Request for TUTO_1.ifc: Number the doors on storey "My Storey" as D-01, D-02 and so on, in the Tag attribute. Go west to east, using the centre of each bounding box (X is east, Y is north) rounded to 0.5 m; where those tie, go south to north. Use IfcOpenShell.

First a look at what the model holds.

```python
import ifcopenshell
import ifcopenshell.util.element
import ifcopenshell.util.placement

model = ifcopenshell.open("TUTO_1.ifc")
print(model.schema)
storey = next(s for s in model.by_type("IfcBuildingStorey") if s.Name == "My Storey")
doors = [e for e in ifcopenshell.util.element.get_decomposition(storey) if e.is_a("IfcDoor")]
for e in sorted(doors, key=lambda e: e.id()):
    origin = ifcopenshell.util.placement.get_local_placement(e.ObjectPlacement)[:3, 3]
    print(e.id(), e.Tag, e.Name, origin.round(2) + 0.0, sep=" | ")
```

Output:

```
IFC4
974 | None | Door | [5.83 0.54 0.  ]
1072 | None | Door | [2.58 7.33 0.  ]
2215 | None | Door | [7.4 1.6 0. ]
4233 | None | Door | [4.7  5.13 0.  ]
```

```python
import ifcopenshell
import ifcopenshell.geom
import ifcopenshell.util.element
import ifcopenshell.util.shape

model = ifcopenshell.open("TUTO_1.ifc")
settings = ifcopenshell.geom.settings()
settings.set("use-world-coords", True)


def centre(element):
    shape = ifcopenshell.geom.create_shape(settings, element)
    return ifcopenshell.util.shape.get_bbox_centroid(shape.geometry)


storey = next(s for s in model.by_type("IfcBuildingStorey") if s.Name == "My Storey")
doors = [e for e in ifcopenshell.util.element.get_decomposition(storey) if e.is_a("IfcDoor")]

# Insertion points can sit at a corner or the storey origin, so sort by the geometry (in metres).
centres = {e: centre(e) for e in doors}
doors.sort(key=lambda e: (round(centres[e][0] / 0.5), centres[e][1]))

for i, e in enumerate(doors, start=1):
    number = f"D-{i:02d}"
    e.Tag = number
    print(e.id(), number)

model.write("TUTO_1-out.ifc")
```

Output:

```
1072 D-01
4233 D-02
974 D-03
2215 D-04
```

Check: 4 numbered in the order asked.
